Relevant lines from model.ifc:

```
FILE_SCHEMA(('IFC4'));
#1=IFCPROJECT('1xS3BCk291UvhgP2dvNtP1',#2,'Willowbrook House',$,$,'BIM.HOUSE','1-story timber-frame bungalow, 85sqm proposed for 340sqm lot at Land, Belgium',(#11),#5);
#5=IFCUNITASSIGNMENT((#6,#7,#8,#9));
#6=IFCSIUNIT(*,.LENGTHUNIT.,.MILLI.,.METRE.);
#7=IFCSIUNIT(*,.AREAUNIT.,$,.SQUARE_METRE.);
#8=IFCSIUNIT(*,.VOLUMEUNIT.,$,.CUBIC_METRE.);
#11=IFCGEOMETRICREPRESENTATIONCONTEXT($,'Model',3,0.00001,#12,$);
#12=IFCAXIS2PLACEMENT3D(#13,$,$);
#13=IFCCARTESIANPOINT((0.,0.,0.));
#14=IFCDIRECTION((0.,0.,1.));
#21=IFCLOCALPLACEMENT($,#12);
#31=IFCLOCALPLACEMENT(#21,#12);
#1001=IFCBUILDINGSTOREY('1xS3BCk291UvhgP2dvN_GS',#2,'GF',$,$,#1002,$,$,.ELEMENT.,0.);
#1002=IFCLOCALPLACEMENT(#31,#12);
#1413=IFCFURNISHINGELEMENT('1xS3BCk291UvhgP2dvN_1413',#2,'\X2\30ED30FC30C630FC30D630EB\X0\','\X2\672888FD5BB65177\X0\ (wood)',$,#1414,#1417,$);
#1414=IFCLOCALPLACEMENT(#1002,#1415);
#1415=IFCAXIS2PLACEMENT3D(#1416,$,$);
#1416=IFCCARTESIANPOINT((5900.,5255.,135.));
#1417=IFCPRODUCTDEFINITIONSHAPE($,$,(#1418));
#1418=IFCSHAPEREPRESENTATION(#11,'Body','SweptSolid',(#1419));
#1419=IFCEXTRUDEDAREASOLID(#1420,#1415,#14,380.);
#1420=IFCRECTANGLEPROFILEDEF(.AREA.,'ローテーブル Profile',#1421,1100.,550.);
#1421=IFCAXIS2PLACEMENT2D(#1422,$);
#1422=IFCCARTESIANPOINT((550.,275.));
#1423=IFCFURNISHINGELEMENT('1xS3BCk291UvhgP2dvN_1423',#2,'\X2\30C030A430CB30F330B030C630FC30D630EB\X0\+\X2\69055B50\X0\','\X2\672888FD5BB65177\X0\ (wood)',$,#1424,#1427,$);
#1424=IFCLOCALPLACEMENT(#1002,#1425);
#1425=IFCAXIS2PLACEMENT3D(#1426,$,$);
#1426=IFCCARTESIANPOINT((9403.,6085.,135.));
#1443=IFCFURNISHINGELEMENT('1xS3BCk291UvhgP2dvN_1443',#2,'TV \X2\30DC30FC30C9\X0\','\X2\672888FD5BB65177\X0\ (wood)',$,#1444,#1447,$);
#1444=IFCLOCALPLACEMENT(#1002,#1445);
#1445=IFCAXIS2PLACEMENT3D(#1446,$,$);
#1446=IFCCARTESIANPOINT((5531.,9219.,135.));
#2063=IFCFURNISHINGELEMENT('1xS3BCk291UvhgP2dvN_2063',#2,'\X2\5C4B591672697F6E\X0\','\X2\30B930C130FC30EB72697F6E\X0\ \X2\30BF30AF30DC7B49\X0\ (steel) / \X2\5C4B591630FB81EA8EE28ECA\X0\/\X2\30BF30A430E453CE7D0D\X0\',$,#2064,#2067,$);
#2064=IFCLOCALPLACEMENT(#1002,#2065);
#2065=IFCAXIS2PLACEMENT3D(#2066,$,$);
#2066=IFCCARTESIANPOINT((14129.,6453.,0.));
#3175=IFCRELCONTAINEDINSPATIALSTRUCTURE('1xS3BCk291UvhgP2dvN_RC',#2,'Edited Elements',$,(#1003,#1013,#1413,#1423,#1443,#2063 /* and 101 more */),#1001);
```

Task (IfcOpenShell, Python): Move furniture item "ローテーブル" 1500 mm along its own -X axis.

```python
import ifcopenshell
import ifcopenshell.api.geometry
import ifcopenshell.util.placement
import ifcopenshell.util.unit

model = ifcopenshell.open("model.ifc")
unit_scale = ifcopenshell.util.unit.calculate_unit_scale(model)

item = model.by_guid("1xS3BCk291UvhgP2dvN_1413")
matrix = ifcopenshell.util.placement.get_local_placement(item.ObjectPlacement)
matrix[:3, 3] -= matrix[:3, 0] * 1.5 / unit_scale
ifcopenshell.api.geometry.edit_object_placement(model, product=item, matrix=matrix, is_si=False)

print(ifcopenshell.util.placement.get_local_placement(item.ObjectPlacement).round(3) + 0.0)

model.write("model_v2.ifc")
```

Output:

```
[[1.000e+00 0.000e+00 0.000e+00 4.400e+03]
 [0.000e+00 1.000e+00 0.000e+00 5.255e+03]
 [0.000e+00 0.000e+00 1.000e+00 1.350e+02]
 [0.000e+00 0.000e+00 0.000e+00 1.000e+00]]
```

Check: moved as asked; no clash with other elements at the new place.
